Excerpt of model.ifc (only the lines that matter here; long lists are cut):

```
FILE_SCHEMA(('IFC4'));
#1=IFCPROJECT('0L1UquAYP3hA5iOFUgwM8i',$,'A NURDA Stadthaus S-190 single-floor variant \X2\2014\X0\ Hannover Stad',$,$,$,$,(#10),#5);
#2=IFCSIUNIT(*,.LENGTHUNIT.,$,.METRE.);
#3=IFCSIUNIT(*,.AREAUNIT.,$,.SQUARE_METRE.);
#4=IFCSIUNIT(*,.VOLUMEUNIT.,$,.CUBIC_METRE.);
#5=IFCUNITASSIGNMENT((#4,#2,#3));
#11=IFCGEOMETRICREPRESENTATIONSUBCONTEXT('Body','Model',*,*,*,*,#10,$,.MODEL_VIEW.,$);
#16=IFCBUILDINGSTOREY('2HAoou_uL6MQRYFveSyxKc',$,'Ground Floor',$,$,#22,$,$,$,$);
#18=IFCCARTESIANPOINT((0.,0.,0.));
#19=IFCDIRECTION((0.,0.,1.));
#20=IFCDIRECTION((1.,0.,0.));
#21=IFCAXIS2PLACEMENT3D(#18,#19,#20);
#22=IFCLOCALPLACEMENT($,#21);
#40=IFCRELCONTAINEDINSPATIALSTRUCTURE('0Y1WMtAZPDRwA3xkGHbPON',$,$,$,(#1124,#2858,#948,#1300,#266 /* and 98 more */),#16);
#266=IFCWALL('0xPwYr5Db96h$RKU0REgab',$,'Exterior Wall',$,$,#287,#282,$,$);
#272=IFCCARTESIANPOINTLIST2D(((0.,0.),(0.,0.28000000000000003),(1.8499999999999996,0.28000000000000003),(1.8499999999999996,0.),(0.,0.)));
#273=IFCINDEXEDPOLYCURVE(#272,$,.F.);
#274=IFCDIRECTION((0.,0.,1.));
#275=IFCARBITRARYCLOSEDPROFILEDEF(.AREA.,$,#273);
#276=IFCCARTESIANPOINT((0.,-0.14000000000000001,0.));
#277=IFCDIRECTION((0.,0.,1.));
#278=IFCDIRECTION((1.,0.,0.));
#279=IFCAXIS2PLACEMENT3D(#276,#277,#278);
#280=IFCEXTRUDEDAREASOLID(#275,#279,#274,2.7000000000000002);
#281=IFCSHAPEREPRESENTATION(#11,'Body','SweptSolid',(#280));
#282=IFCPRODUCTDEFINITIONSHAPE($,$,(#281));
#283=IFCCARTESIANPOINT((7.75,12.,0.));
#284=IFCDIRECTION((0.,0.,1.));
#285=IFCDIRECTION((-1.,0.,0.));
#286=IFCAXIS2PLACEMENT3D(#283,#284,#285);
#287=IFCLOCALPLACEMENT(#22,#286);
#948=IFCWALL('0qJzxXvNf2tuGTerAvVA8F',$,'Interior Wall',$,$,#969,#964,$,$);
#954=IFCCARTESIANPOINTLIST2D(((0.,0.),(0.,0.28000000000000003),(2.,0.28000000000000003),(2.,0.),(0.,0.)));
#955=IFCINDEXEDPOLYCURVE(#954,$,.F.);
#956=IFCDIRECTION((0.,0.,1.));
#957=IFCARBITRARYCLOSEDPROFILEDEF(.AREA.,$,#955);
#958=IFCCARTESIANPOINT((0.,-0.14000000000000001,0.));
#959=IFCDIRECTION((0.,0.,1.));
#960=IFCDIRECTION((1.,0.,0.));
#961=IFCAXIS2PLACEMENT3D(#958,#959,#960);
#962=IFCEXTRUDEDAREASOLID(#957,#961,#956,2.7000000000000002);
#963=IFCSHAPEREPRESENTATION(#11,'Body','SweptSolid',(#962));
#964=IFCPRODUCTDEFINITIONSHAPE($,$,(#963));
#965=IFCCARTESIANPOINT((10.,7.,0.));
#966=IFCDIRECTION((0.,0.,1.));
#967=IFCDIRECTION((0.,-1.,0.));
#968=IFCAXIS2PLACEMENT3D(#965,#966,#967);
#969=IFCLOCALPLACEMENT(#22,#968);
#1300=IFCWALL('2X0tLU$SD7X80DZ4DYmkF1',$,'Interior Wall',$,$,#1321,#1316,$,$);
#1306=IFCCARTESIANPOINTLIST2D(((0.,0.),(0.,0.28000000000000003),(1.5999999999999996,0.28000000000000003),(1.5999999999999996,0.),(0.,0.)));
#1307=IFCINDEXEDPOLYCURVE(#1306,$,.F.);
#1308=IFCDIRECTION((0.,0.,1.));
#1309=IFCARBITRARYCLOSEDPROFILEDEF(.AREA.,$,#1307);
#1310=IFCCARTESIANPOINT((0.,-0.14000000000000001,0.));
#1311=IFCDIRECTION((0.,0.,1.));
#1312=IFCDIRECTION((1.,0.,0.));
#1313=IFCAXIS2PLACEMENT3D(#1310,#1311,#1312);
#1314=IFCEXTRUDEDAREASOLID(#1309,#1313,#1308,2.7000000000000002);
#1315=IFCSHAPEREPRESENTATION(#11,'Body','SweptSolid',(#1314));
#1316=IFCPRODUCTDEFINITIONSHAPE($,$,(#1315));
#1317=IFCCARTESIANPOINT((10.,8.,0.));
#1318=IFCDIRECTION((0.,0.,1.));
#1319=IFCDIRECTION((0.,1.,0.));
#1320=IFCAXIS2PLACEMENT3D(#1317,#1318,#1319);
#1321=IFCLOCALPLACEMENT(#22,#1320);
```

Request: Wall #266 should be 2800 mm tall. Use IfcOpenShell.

```python
import ifcopenshell
import ifcopenshell.geom
import ifcopenshell.util.representation
import ifcopenshell.util.shape
import ifcopenshell.util.unit

model = ifcopenshell.open("model.ifc")
unit_scale = ifcopenshell.util.unit.calculate_unit_scale(model)
settings = ifcopenshell.geom.settings()


def volume(element):
    """Net volume in cubic metres, openings subtracted."""
    shape = ifcopenshell.geom.create_shape(settings, element)
    return ifcopenshell.util.shape.get_volume(shape.geometry)


wall = model.by_guid("0xPwYr5Db96h$RKU0REgab")
before = volume(wall)

body = ifcopenshell.util.representation.get_representation(wall, "Model", "Body")
solid = body.Items[0]
old_height = solid.Depth
solid.Depth = 2.8 / unit_scale
after = volume(wall)

print(f"height {old_height:g} -> {solid.Depth:g}, volume {before:.3f} -> {after:.3f} m3")

model.write("model_v2.ifc")
```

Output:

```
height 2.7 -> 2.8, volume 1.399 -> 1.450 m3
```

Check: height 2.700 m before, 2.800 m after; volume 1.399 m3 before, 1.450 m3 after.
